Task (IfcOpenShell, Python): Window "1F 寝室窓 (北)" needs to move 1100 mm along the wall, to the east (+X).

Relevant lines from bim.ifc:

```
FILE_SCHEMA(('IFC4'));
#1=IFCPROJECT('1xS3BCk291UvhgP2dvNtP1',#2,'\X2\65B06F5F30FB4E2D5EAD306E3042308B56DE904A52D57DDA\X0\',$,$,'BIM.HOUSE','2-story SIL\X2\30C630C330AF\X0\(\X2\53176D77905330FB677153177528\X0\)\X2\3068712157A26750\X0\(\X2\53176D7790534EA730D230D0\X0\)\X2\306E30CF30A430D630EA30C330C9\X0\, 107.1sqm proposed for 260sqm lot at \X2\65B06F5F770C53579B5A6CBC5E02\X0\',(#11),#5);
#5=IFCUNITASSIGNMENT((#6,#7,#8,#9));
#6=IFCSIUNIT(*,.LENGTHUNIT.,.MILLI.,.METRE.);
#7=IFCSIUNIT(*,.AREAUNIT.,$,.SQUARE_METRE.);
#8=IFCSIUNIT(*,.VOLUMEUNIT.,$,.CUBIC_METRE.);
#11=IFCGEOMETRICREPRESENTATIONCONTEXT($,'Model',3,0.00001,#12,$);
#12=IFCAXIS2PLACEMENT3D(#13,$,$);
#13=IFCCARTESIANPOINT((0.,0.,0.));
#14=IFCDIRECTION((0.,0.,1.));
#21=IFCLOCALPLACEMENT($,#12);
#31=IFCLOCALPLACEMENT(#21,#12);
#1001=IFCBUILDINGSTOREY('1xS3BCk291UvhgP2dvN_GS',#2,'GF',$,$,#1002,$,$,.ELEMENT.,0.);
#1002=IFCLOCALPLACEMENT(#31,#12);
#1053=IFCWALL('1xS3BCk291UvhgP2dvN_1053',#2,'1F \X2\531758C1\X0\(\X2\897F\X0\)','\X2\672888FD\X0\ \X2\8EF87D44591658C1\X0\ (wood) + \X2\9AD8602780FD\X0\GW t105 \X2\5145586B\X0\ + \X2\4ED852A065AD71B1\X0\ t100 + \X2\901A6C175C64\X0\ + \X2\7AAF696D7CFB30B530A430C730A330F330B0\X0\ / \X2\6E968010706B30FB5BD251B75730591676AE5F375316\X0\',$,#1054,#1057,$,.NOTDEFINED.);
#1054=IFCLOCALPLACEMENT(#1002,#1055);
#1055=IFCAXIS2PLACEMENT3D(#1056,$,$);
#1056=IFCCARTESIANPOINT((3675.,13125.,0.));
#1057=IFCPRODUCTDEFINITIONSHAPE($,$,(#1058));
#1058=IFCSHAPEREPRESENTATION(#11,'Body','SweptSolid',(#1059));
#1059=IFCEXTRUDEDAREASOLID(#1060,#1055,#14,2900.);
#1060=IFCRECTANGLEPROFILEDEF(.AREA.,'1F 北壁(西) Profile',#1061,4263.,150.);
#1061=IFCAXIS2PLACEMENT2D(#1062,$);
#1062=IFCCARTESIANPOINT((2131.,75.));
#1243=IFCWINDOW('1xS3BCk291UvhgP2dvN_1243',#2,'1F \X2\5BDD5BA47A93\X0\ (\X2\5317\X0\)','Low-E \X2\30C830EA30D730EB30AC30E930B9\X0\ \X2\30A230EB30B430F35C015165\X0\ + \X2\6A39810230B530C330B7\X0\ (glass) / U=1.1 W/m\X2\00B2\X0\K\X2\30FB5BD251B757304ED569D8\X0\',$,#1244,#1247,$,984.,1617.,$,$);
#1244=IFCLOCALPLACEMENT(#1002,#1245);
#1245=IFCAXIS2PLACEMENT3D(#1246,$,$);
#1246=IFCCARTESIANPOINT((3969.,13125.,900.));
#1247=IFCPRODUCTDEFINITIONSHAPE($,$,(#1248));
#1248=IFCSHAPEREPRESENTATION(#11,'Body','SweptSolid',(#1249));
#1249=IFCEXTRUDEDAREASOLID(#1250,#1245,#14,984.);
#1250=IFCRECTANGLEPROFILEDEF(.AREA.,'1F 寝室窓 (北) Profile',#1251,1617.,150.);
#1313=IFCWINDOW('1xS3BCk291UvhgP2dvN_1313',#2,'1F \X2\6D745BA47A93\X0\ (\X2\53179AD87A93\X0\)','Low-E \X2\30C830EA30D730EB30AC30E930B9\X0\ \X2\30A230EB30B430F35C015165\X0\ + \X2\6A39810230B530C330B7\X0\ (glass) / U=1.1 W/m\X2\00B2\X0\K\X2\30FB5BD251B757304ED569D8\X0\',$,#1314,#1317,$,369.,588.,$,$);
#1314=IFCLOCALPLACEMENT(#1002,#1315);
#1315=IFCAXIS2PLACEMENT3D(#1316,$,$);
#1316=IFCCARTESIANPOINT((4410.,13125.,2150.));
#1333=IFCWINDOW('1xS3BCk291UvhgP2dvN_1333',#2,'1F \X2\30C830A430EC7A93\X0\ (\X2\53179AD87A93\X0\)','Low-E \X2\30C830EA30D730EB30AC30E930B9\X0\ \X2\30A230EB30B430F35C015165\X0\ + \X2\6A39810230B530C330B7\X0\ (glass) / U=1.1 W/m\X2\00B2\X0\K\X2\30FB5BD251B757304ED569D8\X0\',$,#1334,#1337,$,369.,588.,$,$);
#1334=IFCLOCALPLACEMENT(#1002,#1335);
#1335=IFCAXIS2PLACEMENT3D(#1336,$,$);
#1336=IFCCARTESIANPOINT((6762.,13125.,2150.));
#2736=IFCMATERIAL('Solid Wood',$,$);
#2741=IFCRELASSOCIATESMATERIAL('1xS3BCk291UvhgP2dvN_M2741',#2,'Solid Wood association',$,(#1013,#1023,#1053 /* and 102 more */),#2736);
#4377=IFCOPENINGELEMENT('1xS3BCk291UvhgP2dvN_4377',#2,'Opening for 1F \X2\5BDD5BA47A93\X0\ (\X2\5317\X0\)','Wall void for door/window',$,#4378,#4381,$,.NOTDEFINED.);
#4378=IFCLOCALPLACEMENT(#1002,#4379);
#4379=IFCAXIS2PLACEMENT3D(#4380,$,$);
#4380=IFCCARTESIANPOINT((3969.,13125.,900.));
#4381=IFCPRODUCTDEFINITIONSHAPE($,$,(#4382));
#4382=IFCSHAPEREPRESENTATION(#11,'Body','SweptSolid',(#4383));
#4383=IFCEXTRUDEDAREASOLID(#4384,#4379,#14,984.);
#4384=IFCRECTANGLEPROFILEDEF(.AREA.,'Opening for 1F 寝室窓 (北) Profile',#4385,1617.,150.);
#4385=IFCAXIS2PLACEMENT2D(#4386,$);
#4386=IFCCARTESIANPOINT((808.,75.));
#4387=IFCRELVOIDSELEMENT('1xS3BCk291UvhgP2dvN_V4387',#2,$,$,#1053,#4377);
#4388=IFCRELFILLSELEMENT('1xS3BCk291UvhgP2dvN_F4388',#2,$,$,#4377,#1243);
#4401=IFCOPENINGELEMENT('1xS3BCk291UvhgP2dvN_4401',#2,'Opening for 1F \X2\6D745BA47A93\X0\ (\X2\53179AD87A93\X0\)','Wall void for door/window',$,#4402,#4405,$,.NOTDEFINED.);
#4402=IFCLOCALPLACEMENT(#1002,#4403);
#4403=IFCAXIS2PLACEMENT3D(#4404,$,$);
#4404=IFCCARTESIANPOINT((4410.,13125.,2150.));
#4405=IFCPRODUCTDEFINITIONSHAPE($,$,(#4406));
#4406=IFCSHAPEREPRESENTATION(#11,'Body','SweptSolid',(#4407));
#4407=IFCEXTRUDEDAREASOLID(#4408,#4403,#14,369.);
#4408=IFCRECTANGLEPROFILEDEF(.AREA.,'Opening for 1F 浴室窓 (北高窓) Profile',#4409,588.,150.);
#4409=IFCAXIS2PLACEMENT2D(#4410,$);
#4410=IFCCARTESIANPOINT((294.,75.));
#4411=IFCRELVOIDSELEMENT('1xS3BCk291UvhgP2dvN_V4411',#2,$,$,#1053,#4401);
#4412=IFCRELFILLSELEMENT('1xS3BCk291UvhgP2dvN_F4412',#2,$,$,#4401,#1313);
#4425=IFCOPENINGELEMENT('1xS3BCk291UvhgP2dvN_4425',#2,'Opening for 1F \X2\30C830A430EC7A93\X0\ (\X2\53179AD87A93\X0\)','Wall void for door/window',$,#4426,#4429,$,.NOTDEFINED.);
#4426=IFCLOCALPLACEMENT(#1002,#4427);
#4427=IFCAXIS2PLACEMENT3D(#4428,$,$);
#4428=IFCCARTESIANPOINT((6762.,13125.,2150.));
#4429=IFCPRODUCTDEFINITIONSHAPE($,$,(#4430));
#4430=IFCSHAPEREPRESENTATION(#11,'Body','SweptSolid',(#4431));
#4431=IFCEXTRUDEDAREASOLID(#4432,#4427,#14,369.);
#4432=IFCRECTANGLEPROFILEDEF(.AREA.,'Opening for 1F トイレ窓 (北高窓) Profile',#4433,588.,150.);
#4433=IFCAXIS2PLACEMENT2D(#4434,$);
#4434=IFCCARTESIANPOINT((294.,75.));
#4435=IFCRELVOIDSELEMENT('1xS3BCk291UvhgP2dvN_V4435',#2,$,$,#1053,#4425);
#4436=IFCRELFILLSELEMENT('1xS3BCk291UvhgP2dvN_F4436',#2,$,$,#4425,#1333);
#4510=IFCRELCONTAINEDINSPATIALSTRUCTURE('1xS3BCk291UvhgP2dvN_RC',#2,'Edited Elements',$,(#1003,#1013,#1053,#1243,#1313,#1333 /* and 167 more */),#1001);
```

```python
import ifcopenshell
import ifcopenshell.api.geometry
import ifcopenshell.util.placement

model = ifcopenshell.open("bim.ifc")

window = model.by_guid("1xS3BCk291UvhgP2dvN_1243")
opening = window.FillsVoids[0].RelatingOpeningElement
wall = opening.VoidsElements[0].RelatingBuildingElement

wall_matrix = ifcopenshell.util.placement.get_local_placement(wall.ObjectPlacement)
shift = wall_matrix[:3, 0] * 1100.0
before = ifcopenshell.util.placement.get_local_placement(window.ObjectPlacement)[:3, 3].copy()

# The window is not placed relative to its opening, so move both.
for product in (opening, window):
    matrix = ifcopenshell.util.placement.get_local_placement(product.ObjectPlacement)
    matrix[:3, 3] += shift
    ifcopenshell.api.geometry.edit_object_placement(model, product=product, matrix=matrix, is_si=False)

after = ifcopenshell.util.placement.get_local_placement(window.ObjectPlacement)[:3, 3]
print("window moved by", (after - before).round(3) + 0.0)

model.write("bim_v2.ifc")
```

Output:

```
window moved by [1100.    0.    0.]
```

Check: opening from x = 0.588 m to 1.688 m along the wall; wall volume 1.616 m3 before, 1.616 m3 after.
